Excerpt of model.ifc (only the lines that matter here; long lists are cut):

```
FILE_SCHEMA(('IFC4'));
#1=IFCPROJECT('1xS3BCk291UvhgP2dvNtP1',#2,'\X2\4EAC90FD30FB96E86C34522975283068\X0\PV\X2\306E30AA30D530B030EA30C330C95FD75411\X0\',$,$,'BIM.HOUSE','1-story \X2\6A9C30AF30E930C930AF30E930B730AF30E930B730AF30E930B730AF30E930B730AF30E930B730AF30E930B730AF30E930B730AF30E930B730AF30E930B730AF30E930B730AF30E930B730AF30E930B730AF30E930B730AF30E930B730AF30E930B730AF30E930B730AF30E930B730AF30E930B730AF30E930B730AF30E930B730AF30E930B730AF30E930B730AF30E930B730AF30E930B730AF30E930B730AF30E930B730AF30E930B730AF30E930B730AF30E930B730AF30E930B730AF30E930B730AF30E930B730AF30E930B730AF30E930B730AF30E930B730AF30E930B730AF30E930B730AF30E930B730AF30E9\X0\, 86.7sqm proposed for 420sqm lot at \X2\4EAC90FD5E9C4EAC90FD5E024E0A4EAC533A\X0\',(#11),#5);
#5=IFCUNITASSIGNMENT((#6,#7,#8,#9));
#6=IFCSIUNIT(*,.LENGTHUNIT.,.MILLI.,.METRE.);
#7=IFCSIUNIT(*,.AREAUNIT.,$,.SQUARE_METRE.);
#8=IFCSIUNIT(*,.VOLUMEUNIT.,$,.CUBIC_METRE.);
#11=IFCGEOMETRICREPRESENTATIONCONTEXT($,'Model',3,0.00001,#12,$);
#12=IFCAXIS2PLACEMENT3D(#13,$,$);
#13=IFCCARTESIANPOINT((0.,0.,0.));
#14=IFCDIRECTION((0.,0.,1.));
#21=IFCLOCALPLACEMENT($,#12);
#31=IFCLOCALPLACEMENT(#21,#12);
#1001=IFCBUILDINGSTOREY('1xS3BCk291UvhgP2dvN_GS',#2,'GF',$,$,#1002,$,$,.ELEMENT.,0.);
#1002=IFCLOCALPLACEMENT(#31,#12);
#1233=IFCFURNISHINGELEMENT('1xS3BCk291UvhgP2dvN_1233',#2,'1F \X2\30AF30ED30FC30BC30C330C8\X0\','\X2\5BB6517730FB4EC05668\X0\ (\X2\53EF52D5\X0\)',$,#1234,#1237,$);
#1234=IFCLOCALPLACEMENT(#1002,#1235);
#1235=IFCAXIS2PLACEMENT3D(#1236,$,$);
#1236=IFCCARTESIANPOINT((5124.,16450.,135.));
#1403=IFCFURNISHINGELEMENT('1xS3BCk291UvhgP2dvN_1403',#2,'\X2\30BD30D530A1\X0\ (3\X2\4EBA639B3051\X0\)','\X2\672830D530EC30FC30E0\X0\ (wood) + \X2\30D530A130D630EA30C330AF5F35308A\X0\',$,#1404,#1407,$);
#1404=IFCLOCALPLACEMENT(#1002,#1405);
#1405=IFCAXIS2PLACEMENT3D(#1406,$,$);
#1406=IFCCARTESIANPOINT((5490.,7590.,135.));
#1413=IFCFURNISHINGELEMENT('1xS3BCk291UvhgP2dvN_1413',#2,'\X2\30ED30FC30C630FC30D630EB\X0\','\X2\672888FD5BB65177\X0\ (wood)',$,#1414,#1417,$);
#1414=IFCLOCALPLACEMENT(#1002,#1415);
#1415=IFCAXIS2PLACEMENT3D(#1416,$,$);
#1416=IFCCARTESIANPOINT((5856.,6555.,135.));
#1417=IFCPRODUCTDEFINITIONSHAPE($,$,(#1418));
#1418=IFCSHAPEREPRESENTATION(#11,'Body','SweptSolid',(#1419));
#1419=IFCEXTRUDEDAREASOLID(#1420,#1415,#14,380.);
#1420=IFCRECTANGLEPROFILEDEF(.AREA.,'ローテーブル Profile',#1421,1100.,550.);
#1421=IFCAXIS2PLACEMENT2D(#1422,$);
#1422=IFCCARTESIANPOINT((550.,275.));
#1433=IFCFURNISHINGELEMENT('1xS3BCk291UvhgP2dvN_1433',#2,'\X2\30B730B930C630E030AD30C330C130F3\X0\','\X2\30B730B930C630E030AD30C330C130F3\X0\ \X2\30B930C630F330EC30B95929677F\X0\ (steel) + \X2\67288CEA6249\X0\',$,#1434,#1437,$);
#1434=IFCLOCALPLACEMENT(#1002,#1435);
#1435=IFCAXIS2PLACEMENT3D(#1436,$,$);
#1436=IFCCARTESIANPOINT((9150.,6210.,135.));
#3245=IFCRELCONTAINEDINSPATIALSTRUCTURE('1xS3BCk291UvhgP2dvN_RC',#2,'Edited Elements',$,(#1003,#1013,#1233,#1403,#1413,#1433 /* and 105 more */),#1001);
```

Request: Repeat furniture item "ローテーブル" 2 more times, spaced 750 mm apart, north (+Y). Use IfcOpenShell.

```python
import numpy as np
import ifcopenshell
import ifcopenshell.api.geometry
import ifcopenshell.api.root
import ifcopenshell.util.element
import ifcopenshell.util.placement
import ifcopenshell.util.unit

model = ifcopenshell.open("model.ifc")
unit_scale = ifcopenshell.util.unit.calculate_unit_scale(model)


def reuse_history(source, copy):
    """copy_class also copies each property set's owner history, people and application; keep the originals."""
    for rel in copy.IsDefinedBy:
        if rel.is_a("IfcRelDefinesByProperties") and (history := rel.RelatingPropertyDefinition.OwnerHistory):
            rel.RelatingPropertyDefinition.OwnerHistory = source.OwnerHistory
            ifcopenshell.util.element.remove_deep2(model, history)


source = model.by_guid("1xS3BCk291UvhgP2dvN_1413")
base = ifcopenshell.util.placement.get_local_placement(source.ObjectPlacement)
step = np.array([0.0, 1.0, 0.0]) * 0.75 / unit_scale

for i in range(1, 3):
    copy = ifcopenshell.api.root.copy_class(model, product=source)
    copy.Representation = ifcopenshell.util.element.copy_deep(
        model, source.Representation, exclude=["IfcGeometricRepresentationContext", "IfcRepresentationMap"]
    )
    reuse_history(source, copy)
    matrix = base.copy()
    matrix[:3, 3] += i * step
    print("added at", matrix[:3, 3].round(3) + 0.0)
    ifcopenshell.api.geometry.edit_object_placement(model, product=copy, matrix=matrix, is_si=False)

model.write("model_rev.ifc")
```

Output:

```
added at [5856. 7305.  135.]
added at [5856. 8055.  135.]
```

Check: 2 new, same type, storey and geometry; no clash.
